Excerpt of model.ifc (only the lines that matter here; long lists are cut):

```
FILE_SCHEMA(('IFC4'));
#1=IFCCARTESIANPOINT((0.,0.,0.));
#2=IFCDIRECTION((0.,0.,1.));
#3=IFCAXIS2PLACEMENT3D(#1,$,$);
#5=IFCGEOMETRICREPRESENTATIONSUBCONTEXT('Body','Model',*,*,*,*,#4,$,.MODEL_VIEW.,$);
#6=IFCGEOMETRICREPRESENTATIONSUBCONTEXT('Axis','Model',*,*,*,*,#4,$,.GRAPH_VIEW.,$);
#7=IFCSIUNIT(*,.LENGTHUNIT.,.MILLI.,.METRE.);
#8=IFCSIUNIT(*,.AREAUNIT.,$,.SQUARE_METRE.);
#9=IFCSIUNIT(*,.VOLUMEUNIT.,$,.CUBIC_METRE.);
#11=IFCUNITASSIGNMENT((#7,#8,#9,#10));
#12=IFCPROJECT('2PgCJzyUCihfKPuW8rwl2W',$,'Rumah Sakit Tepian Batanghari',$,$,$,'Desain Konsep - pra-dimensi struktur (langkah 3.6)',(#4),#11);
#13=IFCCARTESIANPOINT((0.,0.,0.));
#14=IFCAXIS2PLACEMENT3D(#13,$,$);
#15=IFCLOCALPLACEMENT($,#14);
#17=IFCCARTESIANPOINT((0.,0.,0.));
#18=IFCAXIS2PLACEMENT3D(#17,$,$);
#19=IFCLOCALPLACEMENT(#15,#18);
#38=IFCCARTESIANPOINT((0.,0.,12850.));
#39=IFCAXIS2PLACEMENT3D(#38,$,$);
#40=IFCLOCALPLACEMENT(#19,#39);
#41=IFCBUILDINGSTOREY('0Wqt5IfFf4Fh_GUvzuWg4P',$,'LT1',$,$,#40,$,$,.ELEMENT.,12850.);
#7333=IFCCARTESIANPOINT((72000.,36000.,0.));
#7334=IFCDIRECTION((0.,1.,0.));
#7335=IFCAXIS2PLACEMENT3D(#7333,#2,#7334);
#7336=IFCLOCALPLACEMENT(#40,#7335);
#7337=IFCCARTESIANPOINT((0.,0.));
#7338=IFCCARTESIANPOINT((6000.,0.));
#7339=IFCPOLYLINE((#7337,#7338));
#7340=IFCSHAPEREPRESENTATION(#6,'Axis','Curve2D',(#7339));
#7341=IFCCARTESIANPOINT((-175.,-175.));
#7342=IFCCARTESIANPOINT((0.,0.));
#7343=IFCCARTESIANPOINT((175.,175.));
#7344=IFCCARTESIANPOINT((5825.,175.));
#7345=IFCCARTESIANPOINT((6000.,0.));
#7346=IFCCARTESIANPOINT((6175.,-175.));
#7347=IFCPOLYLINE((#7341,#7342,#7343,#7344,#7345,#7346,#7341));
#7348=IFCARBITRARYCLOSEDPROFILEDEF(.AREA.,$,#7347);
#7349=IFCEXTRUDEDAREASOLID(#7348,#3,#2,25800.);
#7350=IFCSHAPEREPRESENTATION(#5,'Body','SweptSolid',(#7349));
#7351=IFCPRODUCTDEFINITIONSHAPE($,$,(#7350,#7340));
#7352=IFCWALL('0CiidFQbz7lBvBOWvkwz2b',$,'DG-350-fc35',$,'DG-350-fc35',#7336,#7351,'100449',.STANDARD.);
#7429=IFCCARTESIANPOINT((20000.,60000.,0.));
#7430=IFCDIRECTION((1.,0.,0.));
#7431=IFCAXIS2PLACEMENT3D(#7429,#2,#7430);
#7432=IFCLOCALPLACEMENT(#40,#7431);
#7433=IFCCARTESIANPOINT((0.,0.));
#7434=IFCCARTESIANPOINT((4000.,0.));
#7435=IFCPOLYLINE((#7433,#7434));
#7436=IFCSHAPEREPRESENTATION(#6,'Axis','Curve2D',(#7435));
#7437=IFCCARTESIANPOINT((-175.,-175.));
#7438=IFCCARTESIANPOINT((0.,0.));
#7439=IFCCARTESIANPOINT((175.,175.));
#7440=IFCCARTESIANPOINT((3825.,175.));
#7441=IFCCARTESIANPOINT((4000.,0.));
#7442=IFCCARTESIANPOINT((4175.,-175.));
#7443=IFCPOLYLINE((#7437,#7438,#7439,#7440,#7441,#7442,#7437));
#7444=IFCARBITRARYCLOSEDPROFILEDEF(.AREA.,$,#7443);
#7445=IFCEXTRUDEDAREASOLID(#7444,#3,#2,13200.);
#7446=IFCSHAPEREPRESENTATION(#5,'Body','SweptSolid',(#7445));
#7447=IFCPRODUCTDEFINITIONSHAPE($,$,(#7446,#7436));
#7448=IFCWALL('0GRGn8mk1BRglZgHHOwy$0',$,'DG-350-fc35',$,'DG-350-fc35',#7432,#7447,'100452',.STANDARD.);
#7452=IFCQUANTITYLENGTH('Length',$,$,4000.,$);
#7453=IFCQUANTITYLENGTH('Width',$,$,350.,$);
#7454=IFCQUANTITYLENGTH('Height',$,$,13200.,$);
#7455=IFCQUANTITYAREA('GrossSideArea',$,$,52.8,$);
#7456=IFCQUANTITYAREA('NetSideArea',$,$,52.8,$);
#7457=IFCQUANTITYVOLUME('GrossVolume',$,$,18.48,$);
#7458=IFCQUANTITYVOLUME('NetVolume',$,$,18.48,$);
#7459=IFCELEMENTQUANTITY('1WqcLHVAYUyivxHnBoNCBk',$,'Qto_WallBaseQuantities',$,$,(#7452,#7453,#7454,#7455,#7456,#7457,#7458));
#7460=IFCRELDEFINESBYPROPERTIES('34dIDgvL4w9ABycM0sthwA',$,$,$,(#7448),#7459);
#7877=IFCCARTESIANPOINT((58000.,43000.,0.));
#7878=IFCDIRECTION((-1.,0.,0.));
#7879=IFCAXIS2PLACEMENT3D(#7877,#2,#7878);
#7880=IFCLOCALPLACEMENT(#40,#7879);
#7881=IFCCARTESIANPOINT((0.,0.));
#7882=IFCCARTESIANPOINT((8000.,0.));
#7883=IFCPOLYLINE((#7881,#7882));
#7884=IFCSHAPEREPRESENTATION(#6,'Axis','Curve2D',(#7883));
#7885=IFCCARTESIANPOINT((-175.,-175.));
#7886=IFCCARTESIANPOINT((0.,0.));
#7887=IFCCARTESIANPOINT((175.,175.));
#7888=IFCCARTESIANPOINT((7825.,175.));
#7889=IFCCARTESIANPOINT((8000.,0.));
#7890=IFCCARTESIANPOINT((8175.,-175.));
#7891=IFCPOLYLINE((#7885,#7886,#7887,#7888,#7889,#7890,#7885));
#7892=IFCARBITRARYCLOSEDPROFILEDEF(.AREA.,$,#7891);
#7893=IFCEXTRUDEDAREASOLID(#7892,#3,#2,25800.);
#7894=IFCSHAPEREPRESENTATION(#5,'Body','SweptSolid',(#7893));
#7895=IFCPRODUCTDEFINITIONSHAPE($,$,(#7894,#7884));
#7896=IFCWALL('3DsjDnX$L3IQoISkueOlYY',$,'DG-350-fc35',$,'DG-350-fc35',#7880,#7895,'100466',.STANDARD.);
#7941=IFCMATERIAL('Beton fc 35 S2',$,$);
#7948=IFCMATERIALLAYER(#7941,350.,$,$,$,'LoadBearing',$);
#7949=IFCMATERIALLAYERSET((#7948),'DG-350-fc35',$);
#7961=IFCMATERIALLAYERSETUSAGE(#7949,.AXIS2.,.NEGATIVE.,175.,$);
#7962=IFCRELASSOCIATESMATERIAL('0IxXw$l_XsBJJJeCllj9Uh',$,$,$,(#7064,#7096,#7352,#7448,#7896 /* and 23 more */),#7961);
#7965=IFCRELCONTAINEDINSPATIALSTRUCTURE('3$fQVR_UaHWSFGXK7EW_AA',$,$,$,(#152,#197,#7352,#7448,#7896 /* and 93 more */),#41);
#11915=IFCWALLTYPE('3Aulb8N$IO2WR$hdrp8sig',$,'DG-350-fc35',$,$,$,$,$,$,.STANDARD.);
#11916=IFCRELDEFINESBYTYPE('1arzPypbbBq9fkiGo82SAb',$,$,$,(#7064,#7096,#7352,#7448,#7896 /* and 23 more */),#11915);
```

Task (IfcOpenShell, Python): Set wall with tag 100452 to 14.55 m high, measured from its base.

```python
import ifcopenshell
import ifcopenshell.api.pset
import ifcopenshell.geom
import ifcopenshell.util.element
import ifcopenshell.util.representation
import ifcopenshell.util.shape
import ifcopenshell.util.unit

model = ifcopenshell.open("model.ifc")
unit_scale = ifcopenshell.util.unit.calculate_unit_scale(model)
area_scale = ifcopenshell.util.unit.calculate_unit_scale(model, "AREAUNIT")
volume_scale = ifcopenshell.util.unit.calculate_unit_scale(model, "VOLUMEUNIT")
settings = ifcopenshell.geom.settings()


def volume(element):
    """Net volume in cubic metres, openings subtracted."""
    shape = ifcopenshell.geom.create_shape(settings, element)
    return ifcopenshell.util.shape.get_volume(shape.geometry)


wall = model.by_id(7448)
before = volume(wall)

body = ifcopenshell.util.representation.get_representation(wall, "Model", "Body")
solid = body.Items[0]
old_height = solid.Depth
solid.Depth = 14.55 / unit_scale
after = volume(wall)
thickness = 0.35  # wall thickness in metres

# Update the stored height, areas and volumes.
qto = model.by_id(ifcopenshell.util.element.get_pset(wall, "Qto_WallBaseQuantities", should_inherit=False)["id"])
ifcopenshell.api.pset.edit_qto(model, qto=qto, properties={
    "Height": solid.Depth,
    "GrossSideArea": ifcopenshell.util.element.get_pset(wall, "Qto_WallBaseQuantities", "GrossSideArea") * solid.Depth / old_height,
    "NetSideArea": after / thickness / area_scale,
    "GrossVolume": ifcopenshell.util.element.get_pset(wall, "Qto_WallBaseQuantities", "GrossVolume") * solid.Depth / old_height,
    "NetVolume": after / volume_scale,
})

print(f"height {old_height:g} -> {solid.Depth:g}, volume {before:.3f} -> {after:.3f} m3")

model.write("model_rev.ifc")
```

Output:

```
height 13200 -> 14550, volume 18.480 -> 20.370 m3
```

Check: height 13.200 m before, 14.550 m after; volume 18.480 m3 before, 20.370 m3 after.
